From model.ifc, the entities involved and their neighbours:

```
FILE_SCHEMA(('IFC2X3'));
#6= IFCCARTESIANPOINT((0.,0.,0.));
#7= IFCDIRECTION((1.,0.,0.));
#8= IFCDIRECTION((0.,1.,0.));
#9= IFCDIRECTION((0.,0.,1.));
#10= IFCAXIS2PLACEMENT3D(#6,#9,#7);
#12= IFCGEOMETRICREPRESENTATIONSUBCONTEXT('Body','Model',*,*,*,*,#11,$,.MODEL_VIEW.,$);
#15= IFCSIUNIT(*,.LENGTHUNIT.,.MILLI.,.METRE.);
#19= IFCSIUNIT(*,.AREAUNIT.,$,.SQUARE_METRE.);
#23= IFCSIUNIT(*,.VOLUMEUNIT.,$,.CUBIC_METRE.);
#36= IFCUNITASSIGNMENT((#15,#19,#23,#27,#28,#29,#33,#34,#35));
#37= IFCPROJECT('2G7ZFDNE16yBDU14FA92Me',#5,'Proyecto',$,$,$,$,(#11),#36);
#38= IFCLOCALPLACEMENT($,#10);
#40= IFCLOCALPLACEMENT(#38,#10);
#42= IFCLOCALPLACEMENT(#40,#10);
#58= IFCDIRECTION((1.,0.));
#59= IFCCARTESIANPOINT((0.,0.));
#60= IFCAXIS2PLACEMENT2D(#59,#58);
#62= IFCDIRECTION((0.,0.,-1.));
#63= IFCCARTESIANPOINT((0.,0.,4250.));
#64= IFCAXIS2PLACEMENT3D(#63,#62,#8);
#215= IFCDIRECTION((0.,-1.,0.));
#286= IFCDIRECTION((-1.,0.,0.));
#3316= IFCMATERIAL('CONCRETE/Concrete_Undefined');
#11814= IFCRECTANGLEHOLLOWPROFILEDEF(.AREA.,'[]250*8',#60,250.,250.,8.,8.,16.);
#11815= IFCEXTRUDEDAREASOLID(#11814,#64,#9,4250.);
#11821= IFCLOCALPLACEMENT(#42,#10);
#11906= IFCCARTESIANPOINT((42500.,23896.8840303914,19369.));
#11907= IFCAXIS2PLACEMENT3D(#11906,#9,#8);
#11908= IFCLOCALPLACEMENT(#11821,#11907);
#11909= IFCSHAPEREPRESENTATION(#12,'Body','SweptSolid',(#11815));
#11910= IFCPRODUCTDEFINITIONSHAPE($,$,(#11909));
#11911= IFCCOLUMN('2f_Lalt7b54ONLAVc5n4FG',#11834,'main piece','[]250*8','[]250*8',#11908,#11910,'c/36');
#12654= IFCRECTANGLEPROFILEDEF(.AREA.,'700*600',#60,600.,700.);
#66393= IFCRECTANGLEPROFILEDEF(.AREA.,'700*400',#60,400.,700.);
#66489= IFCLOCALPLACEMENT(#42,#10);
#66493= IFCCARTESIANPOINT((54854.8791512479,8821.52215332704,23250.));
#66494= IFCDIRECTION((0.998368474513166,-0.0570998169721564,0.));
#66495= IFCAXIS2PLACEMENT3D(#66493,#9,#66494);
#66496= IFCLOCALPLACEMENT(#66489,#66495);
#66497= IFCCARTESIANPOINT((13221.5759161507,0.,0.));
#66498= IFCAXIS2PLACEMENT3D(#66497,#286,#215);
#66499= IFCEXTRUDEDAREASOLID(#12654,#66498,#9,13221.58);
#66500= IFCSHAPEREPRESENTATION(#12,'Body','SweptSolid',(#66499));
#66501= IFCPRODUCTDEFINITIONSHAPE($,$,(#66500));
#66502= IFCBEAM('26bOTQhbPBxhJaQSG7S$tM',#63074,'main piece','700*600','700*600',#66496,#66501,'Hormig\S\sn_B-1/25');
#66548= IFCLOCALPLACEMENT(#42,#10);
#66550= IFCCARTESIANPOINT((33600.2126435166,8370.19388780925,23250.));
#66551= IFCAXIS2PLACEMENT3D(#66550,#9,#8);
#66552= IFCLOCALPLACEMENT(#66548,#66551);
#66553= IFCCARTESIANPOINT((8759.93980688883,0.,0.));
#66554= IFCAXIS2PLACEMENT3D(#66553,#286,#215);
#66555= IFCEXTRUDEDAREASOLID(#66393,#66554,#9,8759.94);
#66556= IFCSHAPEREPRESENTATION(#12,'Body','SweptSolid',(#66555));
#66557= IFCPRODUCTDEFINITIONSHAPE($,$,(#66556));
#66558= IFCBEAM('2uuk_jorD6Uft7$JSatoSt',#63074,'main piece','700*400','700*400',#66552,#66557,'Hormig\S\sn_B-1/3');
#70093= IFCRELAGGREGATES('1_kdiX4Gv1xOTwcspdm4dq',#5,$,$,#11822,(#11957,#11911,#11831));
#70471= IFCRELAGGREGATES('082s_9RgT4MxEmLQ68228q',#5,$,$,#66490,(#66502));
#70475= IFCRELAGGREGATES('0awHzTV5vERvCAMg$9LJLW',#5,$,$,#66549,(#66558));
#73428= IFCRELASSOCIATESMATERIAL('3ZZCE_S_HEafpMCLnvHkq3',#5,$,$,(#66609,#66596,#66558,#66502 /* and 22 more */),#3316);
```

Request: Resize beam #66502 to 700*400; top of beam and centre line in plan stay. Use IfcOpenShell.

```python
import ifcopenshell
import ifcopenshell.util.element
import ifcopenshell.util.representation

model = ifcopenshell.open("model.ifc")

member = model.by_id(66502)
source = next(p for p in model.by_type("IfcRectangleProfileDef") if p.ProfileName == "700*400")

body = ifcopenshell.util.representation.get_representation(member, "Model", "Body")
solid = body.Items[0]
old_profile = solid.SweptArea

# Copy the section's sizes but keep this member's own profile position.
profile = ifcopenshell.util.element.copy(model, source)
# Profiles are centred, so shift by half the change in depth to hold the top.
shift = (old_profile.YDim - profile.YDim) / 2
x, y = old_profile.Position.Location.Coordinates
up = (0.0, 1.0)  # upwards, in the solid's own plane
location = model.createIfcCartesianPoint((x + up[0] * shift, y + up[1] * shift))
profile.Position = model.createIfcAxis2Placement2D(location, old_profile.Position.RefDirection)
solid.SweptArea = profile
if not model.get_total_inverses(old_profile):
    ifcopenshell.util.element.remove_deep2(model, old_profile)
member.Description = member.Description.replace("700*600", "700*400")
member.ObjectType = member.ObjectType.replace("700*600", "700*400")

print(solid.SweptArea)

model.write("model_edited.ifc")
```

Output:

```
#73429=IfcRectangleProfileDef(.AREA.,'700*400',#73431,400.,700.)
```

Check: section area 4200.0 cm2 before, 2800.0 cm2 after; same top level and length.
